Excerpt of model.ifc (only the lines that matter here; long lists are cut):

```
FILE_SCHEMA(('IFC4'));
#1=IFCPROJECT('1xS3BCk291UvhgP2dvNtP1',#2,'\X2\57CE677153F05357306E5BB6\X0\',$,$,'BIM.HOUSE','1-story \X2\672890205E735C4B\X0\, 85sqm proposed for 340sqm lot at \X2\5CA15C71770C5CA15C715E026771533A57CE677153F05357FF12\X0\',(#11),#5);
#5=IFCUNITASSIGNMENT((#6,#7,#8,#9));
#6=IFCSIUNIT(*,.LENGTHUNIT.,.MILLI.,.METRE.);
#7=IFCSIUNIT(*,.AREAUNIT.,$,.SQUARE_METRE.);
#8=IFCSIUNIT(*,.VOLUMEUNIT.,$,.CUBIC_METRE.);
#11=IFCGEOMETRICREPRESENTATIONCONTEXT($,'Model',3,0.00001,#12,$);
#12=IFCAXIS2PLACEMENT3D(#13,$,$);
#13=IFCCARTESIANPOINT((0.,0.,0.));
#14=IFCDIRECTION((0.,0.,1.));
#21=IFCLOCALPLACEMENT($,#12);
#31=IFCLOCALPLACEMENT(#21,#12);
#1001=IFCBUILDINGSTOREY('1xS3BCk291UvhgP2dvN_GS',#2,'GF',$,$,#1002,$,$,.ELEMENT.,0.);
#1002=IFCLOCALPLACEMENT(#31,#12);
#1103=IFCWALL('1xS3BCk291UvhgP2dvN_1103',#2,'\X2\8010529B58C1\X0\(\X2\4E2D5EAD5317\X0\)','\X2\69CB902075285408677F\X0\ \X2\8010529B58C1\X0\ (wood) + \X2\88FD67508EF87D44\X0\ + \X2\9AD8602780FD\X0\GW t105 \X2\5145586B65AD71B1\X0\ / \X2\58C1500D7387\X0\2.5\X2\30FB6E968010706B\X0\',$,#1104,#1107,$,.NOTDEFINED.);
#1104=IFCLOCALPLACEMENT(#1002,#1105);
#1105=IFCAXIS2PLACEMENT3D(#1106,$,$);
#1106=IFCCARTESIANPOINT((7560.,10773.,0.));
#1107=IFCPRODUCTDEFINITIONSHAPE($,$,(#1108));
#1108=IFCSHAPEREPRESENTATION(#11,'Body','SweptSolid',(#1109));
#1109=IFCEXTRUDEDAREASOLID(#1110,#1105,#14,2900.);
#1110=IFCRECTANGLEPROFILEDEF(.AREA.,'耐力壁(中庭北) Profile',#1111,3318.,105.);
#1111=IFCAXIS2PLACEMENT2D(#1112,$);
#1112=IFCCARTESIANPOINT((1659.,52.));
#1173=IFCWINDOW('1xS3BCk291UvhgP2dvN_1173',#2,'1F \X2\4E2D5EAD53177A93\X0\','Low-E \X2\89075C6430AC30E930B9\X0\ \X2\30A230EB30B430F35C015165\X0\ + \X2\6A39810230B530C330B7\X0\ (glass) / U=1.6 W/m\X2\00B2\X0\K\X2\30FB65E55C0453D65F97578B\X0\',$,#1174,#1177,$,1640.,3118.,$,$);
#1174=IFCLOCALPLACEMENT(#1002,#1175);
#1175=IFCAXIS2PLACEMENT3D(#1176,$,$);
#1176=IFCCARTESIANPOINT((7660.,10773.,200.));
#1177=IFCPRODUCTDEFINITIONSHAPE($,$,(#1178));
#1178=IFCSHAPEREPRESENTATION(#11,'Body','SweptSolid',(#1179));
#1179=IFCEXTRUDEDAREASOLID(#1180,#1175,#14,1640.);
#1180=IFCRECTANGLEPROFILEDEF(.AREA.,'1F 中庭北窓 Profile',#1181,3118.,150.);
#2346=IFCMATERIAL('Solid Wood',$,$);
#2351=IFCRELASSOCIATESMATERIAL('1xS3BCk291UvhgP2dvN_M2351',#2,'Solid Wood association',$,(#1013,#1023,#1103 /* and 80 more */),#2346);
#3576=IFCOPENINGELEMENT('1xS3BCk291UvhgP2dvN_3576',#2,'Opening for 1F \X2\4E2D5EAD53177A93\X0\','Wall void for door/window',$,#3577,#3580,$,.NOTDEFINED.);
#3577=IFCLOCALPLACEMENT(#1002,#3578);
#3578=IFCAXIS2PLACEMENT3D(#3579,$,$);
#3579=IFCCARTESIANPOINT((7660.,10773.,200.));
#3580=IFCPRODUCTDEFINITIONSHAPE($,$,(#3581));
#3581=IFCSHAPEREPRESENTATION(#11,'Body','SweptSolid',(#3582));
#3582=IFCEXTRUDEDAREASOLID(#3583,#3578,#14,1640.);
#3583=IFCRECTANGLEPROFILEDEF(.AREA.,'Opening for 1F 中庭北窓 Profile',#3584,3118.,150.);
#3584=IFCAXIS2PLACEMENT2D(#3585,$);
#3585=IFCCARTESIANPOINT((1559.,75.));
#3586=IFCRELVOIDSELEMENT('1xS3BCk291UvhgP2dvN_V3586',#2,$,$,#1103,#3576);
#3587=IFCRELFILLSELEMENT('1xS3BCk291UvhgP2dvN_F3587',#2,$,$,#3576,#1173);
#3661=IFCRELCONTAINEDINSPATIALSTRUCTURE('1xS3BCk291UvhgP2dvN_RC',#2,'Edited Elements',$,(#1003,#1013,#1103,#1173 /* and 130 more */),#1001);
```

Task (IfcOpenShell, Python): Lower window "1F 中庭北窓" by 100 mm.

```python
import numpy as np
import ifcopenshell
import ifcopenshell.api.geometry
import ifcopenshell.util.placement
import ifcopenshell.util.unit

model = ifcopenshell.open("model.ifc")
unit_scale = ifcopenshell.util.unit.calculate_unit_scale(model)

window = model.by_guid("1xS3BCk291UvhgP2dvN_1173")
opening = window.FillsVoids[0].RelatingOpeningElement
dz = -0.1 / unit_scale

shift = np.array([0.0, 0.0, dz])
# The window is not placed relative to its opening, so move both.
for product in (opening, window):
    matrix = ifcopenshell.util.placement.get_local_placement(product.ObjectPlacement)
    matrix[:3, 3] += shift
    ifcopenshell.api.geometry.edit_object_placement(model, product=product, matrix=matrix, is_si=False)

print(f"moved by {dz * unit_scale:+.3f} m")

model.write("model-out.ifc")
```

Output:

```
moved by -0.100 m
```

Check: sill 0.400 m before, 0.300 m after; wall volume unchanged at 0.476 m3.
